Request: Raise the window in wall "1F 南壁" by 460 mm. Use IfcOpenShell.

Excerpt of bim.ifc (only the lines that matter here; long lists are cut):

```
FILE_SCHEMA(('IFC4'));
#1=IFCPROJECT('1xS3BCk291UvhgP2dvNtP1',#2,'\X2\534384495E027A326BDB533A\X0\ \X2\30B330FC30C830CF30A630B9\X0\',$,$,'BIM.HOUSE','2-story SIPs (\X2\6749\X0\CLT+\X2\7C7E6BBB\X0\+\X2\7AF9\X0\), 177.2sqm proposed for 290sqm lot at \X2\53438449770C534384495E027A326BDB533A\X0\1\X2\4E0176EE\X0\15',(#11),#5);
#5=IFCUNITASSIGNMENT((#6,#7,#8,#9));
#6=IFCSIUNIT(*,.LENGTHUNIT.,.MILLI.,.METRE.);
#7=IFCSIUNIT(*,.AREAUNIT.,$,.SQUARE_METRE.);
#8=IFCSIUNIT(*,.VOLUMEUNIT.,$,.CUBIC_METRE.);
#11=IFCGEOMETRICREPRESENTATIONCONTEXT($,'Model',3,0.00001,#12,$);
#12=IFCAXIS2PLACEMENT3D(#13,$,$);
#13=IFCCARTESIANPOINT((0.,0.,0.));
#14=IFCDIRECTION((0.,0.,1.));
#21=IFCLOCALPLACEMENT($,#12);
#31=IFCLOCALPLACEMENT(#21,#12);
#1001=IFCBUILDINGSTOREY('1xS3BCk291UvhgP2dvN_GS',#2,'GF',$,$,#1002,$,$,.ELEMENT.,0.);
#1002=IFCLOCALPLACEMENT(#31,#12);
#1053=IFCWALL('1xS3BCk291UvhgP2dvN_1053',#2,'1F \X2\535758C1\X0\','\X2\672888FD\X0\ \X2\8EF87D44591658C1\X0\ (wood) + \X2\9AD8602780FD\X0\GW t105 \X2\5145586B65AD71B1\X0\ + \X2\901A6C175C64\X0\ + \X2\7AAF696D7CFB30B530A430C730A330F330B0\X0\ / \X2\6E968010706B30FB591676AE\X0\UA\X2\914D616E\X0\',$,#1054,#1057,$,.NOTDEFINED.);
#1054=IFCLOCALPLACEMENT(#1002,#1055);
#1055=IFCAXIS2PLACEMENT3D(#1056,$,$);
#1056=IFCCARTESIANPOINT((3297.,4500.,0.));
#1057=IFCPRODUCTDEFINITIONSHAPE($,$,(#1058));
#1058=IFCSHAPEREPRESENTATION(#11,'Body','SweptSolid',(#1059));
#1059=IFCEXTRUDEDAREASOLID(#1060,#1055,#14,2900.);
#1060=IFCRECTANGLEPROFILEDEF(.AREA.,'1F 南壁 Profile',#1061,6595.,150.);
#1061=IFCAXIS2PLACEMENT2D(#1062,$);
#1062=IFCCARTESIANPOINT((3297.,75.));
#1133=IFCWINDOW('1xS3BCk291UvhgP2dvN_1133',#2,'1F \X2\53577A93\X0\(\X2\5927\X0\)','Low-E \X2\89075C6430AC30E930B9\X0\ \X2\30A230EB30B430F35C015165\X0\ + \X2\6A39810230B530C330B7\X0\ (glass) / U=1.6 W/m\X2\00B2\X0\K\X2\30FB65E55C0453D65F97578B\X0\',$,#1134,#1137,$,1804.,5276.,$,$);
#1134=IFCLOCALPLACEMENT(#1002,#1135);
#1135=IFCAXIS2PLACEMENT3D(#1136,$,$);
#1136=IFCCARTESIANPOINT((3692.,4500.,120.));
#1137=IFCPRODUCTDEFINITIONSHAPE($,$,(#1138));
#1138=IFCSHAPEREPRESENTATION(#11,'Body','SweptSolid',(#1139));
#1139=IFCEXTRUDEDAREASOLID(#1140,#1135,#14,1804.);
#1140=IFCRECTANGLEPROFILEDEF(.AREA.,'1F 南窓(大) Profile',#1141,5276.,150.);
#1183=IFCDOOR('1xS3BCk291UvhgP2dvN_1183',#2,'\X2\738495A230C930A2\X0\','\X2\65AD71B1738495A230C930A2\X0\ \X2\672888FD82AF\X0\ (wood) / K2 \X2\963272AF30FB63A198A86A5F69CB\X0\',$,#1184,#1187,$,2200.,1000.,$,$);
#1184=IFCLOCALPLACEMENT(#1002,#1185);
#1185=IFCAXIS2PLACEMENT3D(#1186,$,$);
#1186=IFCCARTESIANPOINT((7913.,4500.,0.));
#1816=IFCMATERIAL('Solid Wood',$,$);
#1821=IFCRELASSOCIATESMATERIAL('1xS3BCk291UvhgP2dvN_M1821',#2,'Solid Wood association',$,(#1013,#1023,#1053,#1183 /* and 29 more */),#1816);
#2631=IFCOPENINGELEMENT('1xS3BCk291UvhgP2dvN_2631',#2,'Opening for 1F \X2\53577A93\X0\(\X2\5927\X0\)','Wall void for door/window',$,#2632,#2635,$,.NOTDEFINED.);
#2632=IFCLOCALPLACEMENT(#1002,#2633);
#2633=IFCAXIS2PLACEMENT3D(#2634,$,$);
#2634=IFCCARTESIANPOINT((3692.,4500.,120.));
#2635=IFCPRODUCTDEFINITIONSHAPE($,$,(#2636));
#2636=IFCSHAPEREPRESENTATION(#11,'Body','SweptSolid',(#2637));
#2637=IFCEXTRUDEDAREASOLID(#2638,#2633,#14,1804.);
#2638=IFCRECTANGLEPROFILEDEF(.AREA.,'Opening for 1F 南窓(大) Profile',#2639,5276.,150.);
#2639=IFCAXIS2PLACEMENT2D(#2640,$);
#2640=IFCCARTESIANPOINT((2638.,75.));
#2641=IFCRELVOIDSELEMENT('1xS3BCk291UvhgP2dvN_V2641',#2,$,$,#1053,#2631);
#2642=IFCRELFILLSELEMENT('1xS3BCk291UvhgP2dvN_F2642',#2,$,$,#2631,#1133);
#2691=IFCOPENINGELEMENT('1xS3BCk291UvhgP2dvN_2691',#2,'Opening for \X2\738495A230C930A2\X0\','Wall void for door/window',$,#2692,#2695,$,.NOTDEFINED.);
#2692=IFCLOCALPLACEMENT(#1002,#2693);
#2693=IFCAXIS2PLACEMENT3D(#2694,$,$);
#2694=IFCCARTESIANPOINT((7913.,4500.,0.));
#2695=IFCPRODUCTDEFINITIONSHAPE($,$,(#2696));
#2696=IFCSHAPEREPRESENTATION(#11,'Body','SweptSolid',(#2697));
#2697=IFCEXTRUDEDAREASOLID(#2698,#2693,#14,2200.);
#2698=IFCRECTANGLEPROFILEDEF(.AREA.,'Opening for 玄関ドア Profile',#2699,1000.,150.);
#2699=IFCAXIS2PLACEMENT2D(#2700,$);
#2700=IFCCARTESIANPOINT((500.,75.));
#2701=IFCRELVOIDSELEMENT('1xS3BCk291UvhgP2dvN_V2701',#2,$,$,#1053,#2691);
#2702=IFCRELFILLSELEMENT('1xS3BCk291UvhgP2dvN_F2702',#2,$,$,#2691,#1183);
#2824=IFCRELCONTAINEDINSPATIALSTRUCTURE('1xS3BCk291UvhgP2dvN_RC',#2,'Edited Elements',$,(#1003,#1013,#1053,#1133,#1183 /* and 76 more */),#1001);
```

```python
import numpy as np
import ifcopenshell
import ifcopenshell.api.geometry
import ifcopenshell.util.placement
import ifcopenshell.util.unit

model = ifcopenshell.open("bim.ifc")
unit_scale = ifcopenshell.util.unit.calculate_unit_scale(model)

window = model.by_guid("1xS3BCk291UvhgP2dvN_1133")
opening = window.FillsVoids[0].RelatingOpeningElement
dz = 0.46 / unit_scale

shift = np.array([0.0, 0.0, dz])
# The window is not placed relative to its opening, so move both.
for product in (opening, window):
    matrix = ifcopenshell.util.placement.get_local_placement(product.ObjectPlacement)
    matrix[:3, 3] += shift
    ifcopenshell.api.geometry.edit_object_placement(model, product=product, matrix=matrix, is_si=False)

print(f"moved by {dz * unit_scale:+.3f} m")

model.write("bim_v2.ifc")
```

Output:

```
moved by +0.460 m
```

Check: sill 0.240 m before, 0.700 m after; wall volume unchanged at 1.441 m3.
